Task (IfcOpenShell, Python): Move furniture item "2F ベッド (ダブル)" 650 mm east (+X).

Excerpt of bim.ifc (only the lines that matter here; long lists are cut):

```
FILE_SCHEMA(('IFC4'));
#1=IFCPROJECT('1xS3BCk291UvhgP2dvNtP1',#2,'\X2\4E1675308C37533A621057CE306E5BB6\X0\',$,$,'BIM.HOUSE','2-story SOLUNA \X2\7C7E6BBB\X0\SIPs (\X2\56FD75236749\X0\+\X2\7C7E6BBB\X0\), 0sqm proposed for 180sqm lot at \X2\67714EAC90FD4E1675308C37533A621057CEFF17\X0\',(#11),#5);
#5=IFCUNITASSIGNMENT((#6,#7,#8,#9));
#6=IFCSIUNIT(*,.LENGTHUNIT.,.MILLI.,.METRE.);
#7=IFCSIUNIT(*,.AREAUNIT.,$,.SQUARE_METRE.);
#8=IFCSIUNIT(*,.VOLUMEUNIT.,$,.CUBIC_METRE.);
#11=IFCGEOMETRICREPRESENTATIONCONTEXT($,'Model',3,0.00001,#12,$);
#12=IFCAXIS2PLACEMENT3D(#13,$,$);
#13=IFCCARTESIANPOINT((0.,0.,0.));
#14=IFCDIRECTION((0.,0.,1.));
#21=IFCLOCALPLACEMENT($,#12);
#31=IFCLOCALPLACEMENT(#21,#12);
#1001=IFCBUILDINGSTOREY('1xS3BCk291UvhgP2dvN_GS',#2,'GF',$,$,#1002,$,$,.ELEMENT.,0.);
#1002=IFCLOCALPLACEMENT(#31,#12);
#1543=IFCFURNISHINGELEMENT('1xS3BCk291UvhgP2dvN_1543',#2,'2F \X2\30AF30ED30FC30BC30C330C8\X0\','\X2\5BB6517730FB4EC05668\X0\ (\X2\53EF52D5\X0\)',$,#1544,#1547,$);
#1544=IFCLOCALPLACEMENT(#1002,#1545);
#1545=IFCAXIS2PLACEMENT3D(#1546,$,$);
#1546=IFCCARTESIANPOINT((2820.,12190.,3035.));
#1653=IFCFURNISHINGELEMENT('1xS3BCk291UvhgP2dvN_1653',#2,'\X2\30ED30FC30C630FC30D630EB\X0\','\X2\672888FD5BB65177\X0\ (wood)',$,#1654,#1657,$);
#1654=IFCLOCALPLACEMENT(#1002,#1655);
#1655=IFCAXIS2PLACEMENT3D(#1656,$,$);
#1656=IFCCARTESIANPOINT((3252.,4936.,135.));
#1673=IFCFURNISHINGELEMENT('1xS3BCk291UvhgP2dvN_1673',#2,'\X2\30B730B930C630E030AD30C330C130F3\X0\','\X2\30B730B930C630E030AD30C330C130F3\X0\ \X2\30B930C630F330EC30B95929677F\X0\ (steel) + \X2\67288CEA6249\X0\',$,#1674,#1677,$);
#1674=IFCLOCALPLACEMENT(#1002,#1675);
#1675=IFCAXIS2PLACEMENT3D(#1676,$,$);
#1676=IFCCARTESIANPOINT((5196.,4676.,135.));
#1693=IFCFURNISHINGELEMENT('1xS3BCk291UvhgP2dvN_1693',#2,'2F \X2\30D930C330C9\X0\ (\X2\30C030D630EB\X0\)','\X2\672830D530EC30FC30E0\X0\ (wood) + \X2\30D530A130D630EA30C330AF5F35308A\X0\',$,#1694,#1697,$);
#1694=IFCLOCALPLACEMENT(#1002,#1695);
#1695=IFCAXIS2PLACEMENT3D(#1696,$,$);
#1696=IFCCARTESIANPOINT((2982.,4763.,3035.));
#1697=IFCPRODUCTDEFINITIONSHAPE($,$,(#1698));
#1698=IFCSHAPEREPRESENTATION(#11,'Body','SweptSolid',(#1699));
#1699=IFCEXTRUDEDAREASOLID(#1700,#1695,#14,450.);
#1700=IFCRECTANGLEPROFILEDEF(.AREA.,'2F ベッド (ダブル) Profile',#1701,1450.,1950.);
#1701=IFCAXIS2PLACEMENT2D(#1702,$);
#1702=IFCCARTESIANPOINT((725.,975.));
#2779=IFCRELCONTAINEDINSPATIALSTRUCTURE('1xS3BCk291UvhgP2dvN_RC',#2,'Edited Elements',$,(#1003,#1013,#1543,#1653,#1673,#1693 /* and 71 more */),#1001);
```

```python
import ifcopenshell
import ifcopenshell.api.geometry
import ifcopenshell.util.placement

model = ifcopenshell.open("bim.ifc")

item = model.by_guid("1xS3BCk291UvhgP2dvN_1693")
matrix = ifcopenshell.util.placement.get_local_placement(item.ObjectPlacement)
matrix[0, 3] += 650.0
ifcopenshell.api.geometry.edit_object_placement(model, product=item, matrix=matrix, is_si=False)

print(ifcopenshell.util.placement.get_local_placement(item.ObjectPlacement).round(3) + 0.0)

model.write("bim-out.ifc")
```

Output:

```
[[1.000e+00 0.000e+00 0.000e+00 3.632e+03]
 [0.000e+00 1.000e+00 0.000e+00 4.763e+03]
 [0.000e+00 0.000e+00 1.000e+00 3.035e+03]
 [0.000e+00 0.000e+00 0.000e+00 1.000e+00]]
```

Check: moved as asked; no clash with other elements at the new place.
